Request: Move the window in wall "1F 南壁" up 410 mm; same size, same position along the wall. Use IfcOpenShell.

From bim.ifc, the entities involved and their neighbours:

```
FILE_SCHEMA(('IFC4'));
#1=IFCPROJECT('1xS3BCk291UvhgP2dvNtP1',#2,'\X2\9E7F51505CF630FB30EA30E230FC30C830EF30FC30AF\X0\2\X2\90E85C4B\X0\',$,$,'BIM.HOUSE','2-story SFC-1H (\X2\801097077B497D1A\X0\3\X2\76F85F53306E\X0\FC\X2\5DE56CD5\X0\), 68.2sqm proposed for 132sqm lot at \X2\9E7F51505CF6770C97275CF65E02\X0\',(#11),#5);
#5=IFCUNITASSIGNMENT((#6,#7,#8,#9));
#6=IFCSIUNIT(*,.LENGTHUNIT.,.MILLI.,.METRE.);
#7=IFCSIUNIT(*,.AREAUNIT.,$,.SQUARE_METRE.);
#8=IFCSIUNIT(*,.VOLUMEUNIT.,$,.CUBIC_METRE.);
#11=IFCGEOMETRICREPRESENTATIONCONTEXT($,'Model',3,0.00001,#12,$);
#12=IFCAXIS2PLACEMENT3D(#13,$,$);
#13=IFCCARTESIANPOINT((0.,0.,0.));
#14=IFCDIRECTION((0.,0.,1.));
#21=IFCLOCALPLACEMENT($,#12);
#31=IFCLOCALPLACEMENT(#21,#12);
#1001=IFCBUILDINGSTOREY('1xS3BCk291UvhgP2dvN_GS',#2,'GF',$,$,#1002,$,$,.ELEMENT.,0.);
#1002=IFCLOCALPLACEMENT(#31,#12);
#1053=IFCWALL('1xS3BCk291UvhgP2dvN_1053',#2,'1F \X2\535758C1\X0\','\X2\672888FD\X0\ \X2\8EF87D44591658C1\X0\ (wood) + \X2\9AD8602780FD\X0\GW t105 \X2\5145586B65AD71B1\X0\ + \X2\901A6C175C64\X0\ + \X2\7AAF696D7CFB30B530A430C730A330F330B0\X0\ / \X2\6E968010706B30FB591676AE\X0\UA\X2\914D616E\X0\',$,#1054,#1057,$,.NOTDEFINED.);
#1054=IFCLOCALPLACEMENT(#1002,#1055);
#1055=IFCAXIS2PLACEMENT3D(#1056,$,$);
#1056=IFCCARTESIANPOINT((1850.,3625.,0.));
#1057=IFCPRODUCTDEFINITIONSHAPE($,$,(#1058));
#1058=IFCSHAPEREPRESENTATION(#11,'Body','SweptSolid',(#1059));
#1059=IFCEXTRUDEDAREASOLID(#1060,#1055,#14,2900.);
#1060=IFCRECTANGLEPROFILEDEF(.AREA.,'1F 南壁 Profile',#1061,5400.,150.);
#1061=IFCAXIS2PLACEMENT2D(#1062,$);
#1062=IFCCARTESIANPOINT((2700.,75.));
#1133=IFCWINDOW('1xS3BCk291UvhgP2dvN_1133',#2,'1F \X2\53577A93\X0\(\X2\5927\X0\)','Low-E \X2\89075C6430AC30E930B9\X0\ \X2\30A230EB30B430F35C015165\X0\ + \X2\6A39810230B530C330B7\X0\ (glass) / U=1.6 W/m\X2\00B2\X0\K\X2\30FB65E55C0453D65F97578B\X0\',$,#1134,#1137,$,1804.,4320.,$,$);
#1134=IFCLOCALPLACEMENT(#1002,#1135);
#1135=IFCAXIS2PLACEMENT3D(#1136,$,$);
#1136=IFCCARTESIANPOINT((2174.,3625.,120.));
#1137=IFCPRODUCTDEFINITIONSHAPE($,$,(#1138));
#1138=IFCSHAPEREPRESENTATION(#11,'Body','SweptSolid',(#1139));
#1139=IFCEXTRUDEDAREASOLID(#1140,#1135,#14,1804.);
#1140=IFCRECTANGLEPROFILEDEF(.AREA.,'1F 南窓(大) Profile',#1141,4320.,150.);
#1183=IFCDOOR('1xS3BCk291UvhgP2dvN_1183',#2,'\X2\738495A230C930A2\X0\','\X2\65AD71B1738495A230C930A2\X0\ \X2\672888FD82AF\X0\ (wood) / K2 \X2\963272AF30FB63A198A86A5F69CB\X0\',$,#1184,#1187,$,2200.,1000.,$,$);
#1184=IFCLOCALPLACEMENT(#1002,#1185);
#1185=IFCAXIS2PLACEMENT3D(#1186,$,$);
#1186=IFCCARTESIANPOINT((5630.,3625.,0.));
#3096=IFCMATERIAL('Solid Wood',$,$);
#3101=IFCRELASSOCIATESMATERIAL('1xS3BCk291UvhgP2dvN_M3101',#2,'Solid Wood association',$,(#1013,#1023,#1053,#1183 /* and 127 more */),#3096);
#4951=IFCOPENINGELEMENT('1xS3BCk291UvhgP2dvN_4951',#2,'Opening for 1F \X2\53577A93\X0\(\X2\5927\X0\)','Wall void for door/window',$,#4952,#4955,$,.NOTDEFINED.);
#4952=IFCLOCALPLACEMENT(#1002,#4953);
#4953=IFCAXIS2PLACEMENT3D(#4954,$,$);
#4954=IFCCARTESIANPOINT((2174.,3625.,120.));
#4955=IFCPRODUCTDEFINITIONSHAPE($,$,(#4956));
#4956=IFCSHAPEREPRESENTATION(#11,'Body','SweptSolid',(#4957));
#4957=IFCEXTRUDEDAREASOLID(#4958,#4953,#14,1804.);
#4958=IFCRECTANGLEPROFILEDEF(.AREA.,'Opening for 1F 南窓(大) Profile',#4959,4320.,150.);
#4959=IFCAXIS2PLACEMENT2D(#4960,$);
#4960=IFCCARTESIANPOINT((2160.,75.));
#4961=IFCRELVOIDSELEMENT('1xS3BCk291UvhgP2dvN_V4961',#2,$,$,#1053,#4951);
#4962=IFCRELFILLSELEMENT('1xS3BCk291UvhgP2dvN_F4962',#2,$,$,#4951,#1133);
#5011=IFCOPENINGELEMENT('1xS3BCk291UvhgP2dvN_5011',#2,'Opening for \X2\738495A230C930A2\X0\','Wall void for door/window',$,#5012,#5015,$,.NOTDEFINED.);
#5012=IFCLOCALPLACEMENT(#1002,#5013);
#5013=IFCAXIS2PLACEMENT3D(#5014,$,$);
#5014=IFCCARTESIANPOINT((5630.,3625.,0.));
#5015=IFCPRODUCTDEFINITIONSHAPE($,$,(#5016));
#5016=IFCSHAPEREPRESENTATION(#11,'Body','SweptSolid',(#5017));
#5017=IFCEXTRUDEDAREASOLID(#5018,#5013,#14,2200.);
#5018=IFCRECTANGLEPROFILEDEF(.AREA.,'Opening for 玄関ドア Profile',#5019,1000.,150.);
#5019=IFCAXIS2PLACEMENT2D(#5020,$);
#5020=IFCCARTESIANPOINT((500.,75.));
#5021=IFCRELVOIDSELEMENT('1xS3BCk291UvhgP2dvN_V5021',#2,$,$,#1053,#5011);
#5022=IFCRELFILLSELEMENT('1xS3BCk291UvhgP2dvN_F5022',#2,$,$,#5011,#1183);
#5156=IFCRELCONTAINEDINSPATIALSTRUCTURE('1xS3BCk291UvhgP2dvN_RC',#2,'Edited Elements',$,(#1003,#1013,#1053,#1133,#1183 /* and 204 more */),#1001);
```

```python
import numpy as np
import ifcopenshell
import ifcopenshell.api.geometry
import ifcopenshell.util.placement
import ifcopenshell.util.unit

model = ifcopenshell.open("bim.ifc")
unit_scale = ifcopenshell.util.unit.calculate_unit_scale(model)

window = model.by_guid("1xS3BCk291UvhgP2dvN_1133")
opening = window.FillsVoids[0].RelatingOpeningElement
dz = 410.0

shift = np.array([0.0, 0.0, dz])
# The window is not placed relative to its opening, so move both.
for product in (opening, window):
    matrix = ifcopenshell.util.placement.get_local_placement(product.ObjectPlacement)
    matrix[:3, 3] += shift
    ifcopenshell.api.geometry.edit_object_placement(model, product=product, matrix=matrix, is_si=False)

print(f"moved by {dz * unit_scale:+.3f} m")

model.write("bim-out.ifc")
```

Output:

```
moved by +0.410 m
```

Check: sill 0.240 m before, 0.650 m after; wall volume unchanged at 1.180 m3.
